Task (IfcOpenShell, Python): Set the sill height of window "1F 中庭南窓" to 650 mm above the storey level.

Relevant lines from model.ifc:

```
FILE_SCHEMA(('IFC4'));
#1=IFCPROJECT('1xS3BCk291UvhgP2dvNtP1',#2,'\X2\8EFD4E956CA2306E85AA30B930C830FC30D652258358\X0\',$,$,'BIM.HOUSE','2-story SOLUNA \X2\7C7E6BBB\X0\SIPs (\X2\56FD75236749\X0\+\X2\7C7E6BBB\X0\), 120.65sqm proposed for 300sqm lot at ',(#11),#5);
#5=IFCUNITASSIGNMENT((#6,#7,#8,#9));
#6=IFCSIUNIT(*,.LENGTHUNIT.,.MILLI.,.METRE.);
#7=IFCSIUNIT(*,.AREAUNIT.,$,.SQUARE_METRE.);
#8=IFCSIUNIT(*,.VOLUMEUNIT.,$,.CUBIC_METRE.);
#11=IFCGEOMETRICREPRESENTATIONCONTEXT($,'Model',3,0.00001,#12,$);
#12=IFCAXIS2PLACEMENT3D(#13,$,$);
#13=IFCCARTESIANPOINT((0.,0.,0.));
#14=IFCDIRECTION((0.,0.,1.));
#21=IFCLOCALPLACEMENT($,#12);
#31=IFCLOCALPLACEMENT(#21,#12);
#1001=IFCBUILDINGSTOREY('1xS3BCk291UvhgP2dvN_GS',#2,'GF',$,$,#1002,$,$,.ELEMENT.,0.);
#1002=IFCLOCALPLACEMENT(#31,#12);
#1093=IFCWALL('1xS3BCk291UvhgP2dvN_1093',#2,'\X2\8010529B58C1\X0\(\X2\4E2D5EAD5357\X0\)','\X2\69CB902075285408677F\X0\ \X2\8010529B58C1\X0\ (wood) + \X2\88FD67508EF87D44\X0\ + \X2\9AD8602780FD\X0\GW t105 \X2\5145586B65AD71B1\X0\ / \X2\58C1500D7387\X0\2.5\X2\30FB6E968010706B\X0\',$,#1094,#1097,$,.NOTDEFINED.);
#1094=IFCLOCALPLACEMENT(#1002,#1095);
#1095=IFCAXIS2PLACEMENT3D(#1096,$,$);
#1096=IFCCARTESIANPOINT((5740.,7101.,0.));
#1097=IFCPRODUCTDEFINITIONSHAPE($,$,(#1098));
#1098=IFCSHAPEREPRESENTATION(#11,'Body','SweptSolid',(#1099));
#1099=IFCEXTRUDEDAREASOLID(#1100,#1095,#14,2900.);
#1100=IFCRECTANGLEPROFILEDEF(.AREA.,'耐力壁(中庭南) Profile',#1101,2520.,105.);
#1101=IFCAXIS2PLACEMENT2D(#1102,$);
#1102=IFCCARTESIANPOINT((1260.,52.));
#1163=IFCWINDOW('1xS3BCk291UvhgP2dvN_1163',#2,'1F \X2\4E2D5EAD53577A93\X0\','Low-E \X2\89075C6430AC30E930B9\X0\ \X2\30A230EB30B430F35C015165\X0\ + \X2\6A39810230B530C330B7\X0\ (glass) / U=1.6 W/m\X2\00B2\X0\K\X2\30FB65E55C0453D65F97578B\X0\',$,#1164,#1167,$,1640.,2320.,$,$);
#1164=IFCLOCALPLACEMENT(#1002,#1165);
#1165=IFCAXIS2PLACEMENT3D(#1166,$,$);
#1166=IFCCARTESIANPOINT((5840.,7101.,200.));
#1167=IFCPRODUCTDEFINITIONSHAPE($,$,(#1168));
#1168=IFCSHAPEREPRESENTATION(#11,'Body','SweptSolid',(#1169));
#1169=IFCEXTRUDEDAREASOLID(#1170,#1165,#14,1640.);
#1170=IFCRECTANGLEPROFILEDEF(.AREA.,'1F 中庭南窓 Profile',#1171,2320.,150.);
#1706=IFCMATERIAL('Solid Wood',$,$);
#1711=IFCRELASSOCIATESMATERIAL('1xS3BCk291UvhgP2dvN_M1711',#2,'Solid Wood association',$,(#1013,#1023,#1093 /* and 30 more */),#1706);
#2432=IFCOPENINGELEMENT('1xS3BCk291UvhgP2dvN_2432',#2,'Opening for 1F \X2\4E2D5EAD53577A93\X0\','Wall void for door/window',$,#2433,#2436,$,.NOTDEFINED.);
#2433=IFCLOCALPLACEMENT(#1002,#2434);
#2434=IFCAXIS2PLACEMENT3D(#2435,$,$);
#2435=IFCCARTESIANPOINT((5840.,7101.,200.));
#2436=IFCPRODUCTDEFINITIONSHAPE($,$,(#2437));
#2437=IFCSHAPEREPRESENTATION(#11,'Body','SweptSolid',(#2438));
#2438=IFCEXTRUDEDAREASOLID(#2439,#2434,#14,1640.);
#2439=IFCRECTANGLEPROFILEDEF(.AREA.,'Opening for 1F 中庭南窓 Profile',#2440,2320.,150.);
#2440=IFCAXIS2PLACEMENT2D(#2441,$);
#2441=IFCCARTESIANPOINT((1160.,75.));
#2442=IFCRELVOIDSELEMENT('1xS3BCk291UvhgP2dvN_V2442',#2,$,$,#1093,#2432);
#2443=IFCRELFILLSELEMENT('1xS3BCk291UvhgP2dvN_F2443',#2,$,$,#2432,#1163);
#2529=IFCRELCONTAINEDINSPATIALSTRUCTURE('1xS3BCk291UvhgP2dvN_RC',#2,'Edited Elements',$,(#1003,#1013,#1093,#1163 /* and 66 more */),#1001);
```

```python
import numpy as np
import ifcopenshell
import ifcopenshell.api.geometry
import ifcopenshell.geom
import ifcopenshell.util.element
import ifcopenshell.util.placement
import ifcopenshell.util.shape
import ifcopenshell.util.unit

model = ifcopenshell.open("model.ifc")
unit_scale = ifcopenshell.util.unit.calculate_unit_scale(model)

window = model.by_guid("1xS3BCk291UvhgP2dvN_1163")
opening = window.FillsVoids[0].RelatingOpeningElement
storey = ifcopenshell.util.element.get_container(window, ifc_class="IfcBuildingStorey")
level = ifcopenshell.util.placement.get_local_placement(storey.ObjectPlacement)[2, 3]

# The opening's origin need not be at the sill, so measure its lowest point.
shape = ifcopenshell.geom.create_shape(ifcopenshell.geom.settings(), opening)
bottom = ifcopenshell.util.shape.get_shape_bottom_elevation(shape, shape.geometry) / unit_scale
dz = level + 0.65 / unit_scale - bottom

shift = np.array([0.0, 0.0, dz])
# The window is not placed relative to its opening, so move both.
for product in (opening, window):
    matrix = ifcopenshell.util.placement.get_local_placement(product.ObjectPlacement)
    matrix[:3, 3] += shift
    ifcopenshell.api.geometry.edit_object_placement(model, product=product, matrix=matrix, is_si=False)

print(f"moved by {dz * unit_scale:+.3f} m")

model.write("model_edited.ifc")
```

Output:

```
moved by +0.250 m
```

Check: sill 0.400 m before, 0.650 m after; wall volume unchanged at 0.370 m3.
